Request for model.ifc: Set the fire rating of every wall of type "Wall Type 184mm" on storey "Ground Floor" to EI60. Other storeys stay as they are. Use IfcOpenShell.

First a look at what the model holds.

```python
import ifcopenshell
import ifcopenshell.util.element

model = ifcopenshell.open("model.ifc")
print(model.schema)
storey = next(s for s in model.by_type("IfcBuildingStorey") if s.Name == "Ground Floor")
walls = [e for e in ifcopenshell.util.element.get_decomposition(storey) if e.is_a("IfcWall")]
seen = {}
for e in walls:
    element_type = ifcopenshell.util.element.get_type(e)
    key = (element_type.Name if element_type != e and element_type else None, ifcopenshell.util.element.get_pset(e, "Pset_WallCommon", "FireRating"))
    seen[key] = seen.get(key, 0) + 1
for (name, value), count in sorted(seen.items(), key=str):
    print(count, "x", name, "|", value)
```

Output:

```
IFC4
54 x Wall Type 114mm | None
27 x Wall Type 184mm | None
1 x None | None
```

```python
import ifcopenshell
import ifcopenshell.api.pset
import ifcopenshell.util.element

model = ifcopenshell.open("model.ifc")

storey = next(s for s in model.by_type("IfcBuildingStorey") if s.Name == "Ground Floor")
walls = [e for e in ifcopenshell.util.element.get_decomposition(storey) if e.is_a("IfcWall")]

count = 0
for e in walls:
    element_type = ifcopenshell.util.element.get_type(e)
    if element_type in (None, e) or element_type.Name != "Wall Type 184mm":
        continue
    # add_pset returns the element's existing set when there is one.
    pset = ifcopenshell.api.pset.add_pset(model, product=e, name="Pset_WallCommon")
    ifcopenshell.api.pset.edit_pset(model, pset=pset, properties={"FireRating": "EI60"})
    count += 1

print(count, "walls updated")

model.write("model_v2.ifc")
```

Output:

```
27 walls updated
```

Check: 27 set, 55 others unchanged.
